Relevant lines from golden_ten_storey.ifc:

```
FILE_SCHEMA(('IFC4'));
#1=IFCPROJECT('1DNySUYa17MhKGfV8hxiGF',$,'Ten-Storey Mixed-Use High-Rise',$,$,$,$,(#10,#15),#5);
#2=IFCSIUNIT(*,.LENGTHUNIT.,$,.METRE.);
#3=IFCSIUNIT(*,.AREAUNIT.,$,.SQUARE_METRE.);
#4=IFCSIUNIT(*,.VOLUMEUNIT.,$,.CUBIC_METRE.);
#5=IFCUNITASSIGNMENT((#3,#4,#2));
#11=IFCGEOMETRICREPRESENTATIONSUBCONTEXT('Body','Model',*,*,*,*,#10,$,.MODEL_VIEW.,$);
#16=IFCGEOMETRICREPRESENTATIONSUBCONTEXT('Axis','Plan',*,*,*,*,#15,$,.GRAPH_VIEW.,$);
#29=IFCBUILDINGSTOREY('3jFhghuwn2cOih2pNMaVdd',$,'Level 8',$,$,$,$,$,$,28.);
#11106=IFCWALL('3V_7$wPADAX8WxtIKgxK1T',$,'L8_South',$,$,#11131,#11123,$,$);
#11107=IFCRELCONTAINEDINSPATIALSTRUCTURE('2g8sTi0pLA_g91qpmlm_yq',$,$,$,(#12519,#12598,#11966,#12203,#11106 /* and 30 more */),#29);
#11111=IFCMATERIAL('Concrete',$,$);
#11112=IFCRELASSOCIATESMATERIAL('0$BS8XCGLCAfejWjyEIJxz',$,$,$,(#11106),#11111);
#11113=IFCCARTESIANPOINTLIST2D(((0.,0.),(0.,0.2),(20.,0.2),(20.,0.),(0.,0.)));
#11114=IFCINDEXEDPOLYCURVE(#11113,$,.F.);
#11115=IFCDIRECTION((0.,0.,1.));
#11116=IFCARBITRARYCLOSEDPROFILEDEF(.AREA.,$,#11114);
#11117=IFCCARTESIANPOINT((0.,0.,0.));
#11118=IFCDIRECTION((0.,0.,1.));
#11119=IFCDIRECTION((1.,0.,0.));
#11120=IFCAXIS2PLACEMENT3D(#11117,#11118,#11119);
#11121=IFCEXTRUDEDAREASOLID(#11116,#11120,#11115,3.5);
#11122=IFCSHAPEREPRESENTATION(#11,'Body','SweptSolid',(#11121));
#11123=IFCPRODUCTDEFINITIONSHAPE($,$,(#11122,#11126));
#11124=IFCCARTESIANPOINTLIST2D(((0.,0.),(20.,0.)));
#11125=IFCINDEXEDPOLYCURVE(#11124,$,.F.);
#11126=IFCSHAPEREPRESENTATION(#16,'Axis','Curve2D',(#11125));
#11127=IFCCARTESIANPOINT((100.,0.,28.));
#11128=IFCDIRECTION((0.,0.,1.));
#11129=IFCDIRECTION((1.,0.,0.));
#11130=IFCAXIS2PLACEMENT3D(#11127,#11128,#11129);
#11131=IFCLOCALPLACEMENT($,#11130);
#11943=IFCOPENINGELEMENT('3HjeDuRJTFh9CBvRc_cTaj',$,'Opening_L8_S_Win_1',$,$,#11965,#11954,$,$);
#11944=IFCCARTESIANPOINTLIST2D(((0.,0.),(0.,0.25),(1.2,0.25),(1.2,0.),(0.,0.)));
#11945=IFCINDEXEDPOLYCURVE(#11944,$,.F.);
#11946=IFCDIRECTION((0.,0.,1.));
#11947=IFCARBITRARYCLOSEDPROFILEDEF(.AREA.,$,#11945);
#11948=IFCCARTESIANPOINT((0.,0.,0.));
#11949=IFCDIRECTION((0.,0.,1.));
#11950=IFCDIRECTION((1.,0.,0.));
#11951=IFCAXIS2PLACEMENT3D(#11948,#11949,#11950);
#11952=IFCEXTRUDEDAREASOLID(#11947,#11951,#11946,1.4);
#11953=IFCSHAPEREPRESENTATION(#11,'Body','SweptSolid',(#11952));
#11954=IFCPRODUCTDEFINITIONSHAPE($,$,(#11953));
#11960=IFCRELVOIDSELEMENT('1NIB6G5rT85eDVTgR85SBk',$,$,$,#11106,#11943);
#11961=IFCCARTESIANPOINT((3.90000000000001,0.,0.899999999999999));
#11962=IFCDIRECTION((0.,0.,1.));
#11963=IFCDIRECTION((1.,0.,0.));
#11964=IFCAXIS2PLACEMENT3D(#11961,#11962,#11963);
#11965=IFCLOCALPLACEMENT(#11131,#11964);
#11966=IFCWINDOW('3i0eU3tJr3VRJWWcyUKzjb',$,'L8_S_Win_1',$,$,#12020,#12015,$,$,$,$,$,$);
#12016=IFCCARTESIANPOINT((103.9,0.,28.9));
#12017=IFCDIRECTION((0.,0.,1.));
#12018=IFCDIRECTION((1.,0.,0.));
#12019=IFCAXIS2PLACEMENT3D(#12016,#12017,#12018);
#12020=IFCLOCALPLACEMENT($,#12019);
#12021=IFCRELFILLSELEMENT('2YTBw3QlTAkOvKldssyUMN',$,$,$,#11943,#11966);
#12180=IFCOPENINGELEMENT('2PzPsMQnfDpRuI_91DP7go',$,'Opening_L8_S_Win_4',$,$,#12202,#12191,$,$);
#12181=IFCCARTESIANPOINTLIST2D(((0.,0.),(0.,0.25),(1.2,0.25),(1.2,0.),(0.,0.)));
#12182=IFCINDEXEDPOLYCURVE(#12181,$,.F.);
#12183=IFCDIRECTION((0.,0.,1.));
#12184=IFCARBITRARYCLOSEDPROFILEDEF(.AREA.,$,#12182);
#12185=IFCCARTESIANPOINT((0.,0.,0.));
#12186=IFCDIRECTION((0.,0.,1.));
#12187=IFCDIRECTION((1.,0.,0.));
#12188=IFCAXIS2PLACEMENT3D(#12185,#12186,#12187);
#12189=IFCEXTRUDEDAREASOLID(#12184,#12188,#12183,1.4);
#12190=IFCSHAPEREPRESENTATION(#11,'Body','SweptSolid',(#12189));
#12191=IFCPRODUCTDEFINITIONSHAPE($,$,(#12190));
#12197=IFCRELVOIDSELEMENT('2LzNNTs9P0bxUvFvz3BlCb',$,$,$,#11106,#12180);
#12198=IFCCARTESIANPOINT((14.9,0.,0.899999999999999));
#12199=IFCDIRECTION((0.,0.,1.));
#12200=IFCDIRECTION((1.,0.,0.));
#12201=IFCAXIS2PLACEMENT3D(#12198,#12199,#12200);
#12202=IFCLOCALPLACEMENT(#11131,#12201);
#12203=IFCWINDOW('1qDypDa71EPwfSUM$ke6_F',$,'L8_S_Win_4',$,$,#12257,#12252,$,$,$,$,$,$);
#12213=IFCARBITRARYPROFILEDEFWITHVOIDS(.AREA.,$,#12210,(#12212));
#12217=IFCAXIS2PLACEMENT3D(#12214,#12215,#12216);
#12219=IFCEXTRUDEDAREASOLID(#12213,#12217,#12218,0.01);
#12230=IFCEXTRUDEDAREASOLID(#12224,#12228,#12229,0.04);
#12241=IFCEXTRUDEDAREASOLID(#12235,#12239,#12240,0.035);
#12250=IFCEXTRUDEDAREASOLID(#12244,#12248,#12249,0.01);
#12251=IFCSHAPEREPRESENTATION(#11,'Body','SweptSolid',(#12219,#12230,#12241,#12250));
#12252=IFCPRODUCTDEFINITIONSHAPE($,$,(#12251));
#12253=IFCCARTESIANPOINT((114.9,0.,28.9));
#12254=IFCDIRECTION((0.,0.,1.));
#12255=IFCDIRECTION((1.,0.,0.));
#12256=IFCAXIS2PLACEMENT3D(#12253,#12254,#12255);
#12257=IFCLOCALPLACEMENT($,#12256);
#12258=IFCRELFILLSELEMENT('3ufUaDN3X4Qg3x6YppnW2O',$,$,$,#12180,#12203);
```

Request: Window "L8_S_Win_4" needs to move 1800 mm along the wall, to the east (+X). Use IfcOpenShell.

```python
import ifcopenshell
import ifcopenshell.api.geometry
import ifcopenshell.util.placement
import ifcopenshell.util.unit

model = ifcopenshell.open("golden_ten_storey.ifc")
unit_scale = ifcopenshell.util.unit.calculate_unit_scale(model)

window = model.by_guid("1qDypDa71EPwfSUM$ke6_F")
opening = window.FillsVoids[0].RelatingOpeningElement
wall = opening.VoidsElements[0].RelatingBuildingElement

wall_matrix = ifcopenshell.util.placement.get_local_placement(wall.ObjectPlacement)
shift = wall_matrix[:3, 0] * 1.8 / unit_scale
before = ifcopenshell.util.placement.get_local_placement(window.ObjectPlacement)[:3, 3].copy()

# The window is not placed relative to its opening, so move both.
for product in (opening, window):
    matrix = ifcopenshell.util.placement.get_local_placement(product.ObjectPlacement)
    matrix[:3, 3] += shift
    ifcopenshell.api.geometry.edit_object_placement(model, product=product, matrix=matrix, is_si=False)

after = ifcopenshell.util.placement.get_local_placement(window.ObjectPlacement)[:3, 3]
print("window moved by", (after - before).round(3) + 0.0)

model.write("golden_ten_storey_v2.ifc")
```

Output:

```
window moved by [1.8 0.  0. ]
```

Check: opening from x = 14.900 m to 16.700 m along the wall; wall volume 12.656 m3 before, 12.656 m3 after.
